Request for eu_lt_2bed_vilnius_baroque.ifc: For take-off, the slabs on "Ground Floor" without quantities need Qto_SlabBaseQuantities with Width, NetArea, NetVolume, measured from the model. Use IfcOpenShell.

First a look at what the model holds.

```python
import ifcopenshell
import ifcopenshell.util.element
import ifcopenshell.util.unit

model = ifcopenshell.open("eu_lt_2bed_vilnius_baroque.ifc")
print(model.schema)
for unit_type in ("LENGTHUNIT", "AREAUNIT", "VOLUMEUNIT"):
    print(unit_type, ifcopenshell.util.unit.calculate_unit_scale(model, unit_type))
storey = next(s for s in model.by_type("IfcBuildingStorey") if s.Name == "Ground Floor")
slabs = [e for e in ifcopenshell.util.element.get_decomposition(storey) if e.is_a("IfcSlab")]
for e in sorted(slabs, key=lambda e: e.id()):
    print(e.id(), e.is_a(), e.Name, list(ifcopenshell.util.element.get_psets(e, qtos_only=True)), sep=" | ")
```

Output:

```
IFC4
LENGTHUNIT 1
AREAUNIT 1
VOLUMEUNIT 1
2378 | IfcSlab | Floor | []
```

```python
import ifcopenshell
import ifcopenshell.api.pset
import ifcopenshell.geom
import ifcopenshell.util.element
import ifcopenshell.util.shape
import ifcopenshell.util.unit

model = ifcopenshell.open("eu_lt_2bed_vilnius_baroque.ifc")
unit_scale = ifcopenshell.util.unit.calculate_unit_scale(model)
area_scale = ifcopenshell.util.unit.calculate_unit_scale(model, "AREAUNIT")
volume_scale = ifcopenshell.util.unit.calculate_unit_scale(model, "VOLUMEUNIT")
settings = ifcopenshell.geom.settings()

storey = next(s for s in model.by_type("IfcBuildingStorey") if s.Name == "Ground Floor")
slabs = [e for e in ifcopenshell.util.element.get_decomposition(storey) if e.is_a("IfcSlab")]

for e in sorted(slabs, key=lambda e: e.id()):
    if ifcopenshell.util.element.get_psets(e, qtos_only=True, should_inherit=False):
        continue
    # Geometry comes back in metres, in the element's own axes.
    shape = ifcopenshell.geom.create_shape(settings, e)
    values = {
        "Width": ifcopenshell.util.shape.get_z(shape.geometry) / unit_scale,
        "NetArea": ifcopenshell.util.shape.get_footprint_area(shape.geometry) / area_scale,
        "NetVolume": ifcopenshell.util.shape.get_volume(shape.geometry) / volume_scale,
    }
    qto = ifcopenshell.api.pset.add_qto(model, product=e, name="Qto_SlabBaseQuantities")
    ifcopenshell.api.pset.edit_qto(model, qto=qto, properties=values)
    print(e.id(), {k: round(v, 3) for k, v in values.items()})

model.write("eu_lt_2bed_vilnius_baroque_updated.ifc")
```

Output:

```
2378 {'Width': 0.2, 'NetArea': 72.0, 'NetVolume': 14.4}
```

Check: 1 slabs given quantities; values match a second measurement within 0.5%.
